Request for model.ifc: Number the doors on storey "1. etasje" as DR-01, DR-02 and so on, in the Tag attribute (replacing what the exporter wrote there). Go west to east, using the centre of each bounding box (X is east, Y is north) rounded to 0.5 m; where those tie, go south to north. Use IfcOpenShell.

First a look at what the model holds.

```python
import ifcopenshell
import ifcopenshell.util.element
import ifcopenshell.util.placement

model = ifcopenshell.open("model.ifc")
print(model.schema)
storey = next(s for s in model.by_type("IfcBuildingStorey") if s.Name == "1. etasje")
doors = [e for e in ifcopenshell.util.element.get_decomposition(storey) if e.is_a("IfcDoor")]
for e in sorted(doors, key=lambda e: e.id()):
    origin = ifcopenshell.util.placement.get_local_placement(e.ObjectPlacement)[:3, 3]
    print(e.id(), e.Tag, e.Name, origin.round(2) + 0.0, sep=" | ")
```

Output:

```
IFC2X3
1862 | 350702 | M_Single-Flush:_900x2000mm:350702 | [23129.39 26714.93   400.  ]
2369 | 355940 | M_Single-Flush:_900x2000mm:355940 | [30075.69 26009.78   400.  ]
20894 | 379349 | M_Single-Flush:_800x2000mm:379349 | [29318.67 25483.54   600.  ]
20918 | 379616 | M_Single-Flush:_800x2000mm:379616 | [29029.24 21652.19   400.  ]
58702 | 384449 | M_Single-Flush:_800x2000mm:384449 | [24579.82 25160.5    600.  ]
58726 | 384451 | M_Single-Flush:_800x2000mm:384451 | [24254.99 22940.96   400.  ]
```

```python
import ifcopenshell
import ifcopenshell.geom
import ifcopenshell.util.element
import ifcopenshell.util.shape

model = ifcopenshell.open("model.ifc")
settings = ifcopenshell.geom.settings()
settings.set("use-world-coords", True)


def centre(element):
    shape = ifcopenshell.geom.create_shape(settings, element)
    return ifcopenshell.util.shape.get_bbox_centroid(shape.geometry)


storey = next(s for s in model.by_type("IfcBuildingStorey") if s.Name == "1. etasje")
doors = [e for e in ifcopenshell.util.element.get_decomposition(storey) if e.is_a("IfcDoor")]

# Insertion points can sit at a corner or the storey origin, so sort by the geometry (in metres).
centres = {e: centre(e) for e in doors}
doors.sort(key=lambda e: (round(centres[e][0] / 0.5), centres[e][1]))

for i, e in enumerate(doors, start=1):
    number = f"DR-{i:02d}"
    e.Tag = number
    print(e.id(), number)

model.write("model_updated.ifc")
```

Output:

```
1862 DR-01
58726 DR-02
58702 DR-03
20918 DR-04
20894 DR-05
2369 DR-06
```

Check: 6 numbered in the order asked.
